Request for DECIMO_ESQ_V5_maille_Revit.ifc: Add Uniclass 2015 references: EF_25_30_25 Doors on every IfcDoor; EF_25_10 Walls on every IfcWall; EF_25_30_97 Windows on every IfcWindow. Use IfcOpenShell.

First a look at what the model holds.

```python
import ifcopenshell

model = ifcopenshell.open("DECIMO_ESQ_V5_maille_Revit.ifc")
print(model.schema)
print("classifications:", [c.Name for c in model.by_type("IfcClassification")])
for ifc_class in ("IfcDoor", "IfcRoof", "IfcStair", "IfcWall", "IfcWindow"):
    print(ifc_class, len(model.by_type(ifc_class)))
```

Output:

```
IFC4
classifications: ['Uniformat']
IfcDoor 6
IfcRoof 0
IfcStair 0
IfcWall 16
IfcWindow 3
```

```python
import ifcopenshell
import ifcopenshell.api.classification

model = ifcopenshell.open("DECIMO_ESQ_V5_maille_Revit.ifc")

system = ifcopenshell.api.classification.add_classification(model, classification="Uniclass 2015")

codes = {
    "IfcDoor": ("EF_25_30_25", "Doors"),
    "IfcWall": ("EF_25_10", "Walls"),
    "IfcWindow": ("EF_25_30_97", "Windows"),
}
for ifc_class, (code, name) in codes.items():
    products = model.by_type(ifc_class)
    ifcopenshell.api.classification.add_reference(
        model, products=products, classification=system, identification=code, name=name
    )
    print(code, len(products))

model.write("DECIMO_ESQ_V5_maille_Revit_v2.ifc")
```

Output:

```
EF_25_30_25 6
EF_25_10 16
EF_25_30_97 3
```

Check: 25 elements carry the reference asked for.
